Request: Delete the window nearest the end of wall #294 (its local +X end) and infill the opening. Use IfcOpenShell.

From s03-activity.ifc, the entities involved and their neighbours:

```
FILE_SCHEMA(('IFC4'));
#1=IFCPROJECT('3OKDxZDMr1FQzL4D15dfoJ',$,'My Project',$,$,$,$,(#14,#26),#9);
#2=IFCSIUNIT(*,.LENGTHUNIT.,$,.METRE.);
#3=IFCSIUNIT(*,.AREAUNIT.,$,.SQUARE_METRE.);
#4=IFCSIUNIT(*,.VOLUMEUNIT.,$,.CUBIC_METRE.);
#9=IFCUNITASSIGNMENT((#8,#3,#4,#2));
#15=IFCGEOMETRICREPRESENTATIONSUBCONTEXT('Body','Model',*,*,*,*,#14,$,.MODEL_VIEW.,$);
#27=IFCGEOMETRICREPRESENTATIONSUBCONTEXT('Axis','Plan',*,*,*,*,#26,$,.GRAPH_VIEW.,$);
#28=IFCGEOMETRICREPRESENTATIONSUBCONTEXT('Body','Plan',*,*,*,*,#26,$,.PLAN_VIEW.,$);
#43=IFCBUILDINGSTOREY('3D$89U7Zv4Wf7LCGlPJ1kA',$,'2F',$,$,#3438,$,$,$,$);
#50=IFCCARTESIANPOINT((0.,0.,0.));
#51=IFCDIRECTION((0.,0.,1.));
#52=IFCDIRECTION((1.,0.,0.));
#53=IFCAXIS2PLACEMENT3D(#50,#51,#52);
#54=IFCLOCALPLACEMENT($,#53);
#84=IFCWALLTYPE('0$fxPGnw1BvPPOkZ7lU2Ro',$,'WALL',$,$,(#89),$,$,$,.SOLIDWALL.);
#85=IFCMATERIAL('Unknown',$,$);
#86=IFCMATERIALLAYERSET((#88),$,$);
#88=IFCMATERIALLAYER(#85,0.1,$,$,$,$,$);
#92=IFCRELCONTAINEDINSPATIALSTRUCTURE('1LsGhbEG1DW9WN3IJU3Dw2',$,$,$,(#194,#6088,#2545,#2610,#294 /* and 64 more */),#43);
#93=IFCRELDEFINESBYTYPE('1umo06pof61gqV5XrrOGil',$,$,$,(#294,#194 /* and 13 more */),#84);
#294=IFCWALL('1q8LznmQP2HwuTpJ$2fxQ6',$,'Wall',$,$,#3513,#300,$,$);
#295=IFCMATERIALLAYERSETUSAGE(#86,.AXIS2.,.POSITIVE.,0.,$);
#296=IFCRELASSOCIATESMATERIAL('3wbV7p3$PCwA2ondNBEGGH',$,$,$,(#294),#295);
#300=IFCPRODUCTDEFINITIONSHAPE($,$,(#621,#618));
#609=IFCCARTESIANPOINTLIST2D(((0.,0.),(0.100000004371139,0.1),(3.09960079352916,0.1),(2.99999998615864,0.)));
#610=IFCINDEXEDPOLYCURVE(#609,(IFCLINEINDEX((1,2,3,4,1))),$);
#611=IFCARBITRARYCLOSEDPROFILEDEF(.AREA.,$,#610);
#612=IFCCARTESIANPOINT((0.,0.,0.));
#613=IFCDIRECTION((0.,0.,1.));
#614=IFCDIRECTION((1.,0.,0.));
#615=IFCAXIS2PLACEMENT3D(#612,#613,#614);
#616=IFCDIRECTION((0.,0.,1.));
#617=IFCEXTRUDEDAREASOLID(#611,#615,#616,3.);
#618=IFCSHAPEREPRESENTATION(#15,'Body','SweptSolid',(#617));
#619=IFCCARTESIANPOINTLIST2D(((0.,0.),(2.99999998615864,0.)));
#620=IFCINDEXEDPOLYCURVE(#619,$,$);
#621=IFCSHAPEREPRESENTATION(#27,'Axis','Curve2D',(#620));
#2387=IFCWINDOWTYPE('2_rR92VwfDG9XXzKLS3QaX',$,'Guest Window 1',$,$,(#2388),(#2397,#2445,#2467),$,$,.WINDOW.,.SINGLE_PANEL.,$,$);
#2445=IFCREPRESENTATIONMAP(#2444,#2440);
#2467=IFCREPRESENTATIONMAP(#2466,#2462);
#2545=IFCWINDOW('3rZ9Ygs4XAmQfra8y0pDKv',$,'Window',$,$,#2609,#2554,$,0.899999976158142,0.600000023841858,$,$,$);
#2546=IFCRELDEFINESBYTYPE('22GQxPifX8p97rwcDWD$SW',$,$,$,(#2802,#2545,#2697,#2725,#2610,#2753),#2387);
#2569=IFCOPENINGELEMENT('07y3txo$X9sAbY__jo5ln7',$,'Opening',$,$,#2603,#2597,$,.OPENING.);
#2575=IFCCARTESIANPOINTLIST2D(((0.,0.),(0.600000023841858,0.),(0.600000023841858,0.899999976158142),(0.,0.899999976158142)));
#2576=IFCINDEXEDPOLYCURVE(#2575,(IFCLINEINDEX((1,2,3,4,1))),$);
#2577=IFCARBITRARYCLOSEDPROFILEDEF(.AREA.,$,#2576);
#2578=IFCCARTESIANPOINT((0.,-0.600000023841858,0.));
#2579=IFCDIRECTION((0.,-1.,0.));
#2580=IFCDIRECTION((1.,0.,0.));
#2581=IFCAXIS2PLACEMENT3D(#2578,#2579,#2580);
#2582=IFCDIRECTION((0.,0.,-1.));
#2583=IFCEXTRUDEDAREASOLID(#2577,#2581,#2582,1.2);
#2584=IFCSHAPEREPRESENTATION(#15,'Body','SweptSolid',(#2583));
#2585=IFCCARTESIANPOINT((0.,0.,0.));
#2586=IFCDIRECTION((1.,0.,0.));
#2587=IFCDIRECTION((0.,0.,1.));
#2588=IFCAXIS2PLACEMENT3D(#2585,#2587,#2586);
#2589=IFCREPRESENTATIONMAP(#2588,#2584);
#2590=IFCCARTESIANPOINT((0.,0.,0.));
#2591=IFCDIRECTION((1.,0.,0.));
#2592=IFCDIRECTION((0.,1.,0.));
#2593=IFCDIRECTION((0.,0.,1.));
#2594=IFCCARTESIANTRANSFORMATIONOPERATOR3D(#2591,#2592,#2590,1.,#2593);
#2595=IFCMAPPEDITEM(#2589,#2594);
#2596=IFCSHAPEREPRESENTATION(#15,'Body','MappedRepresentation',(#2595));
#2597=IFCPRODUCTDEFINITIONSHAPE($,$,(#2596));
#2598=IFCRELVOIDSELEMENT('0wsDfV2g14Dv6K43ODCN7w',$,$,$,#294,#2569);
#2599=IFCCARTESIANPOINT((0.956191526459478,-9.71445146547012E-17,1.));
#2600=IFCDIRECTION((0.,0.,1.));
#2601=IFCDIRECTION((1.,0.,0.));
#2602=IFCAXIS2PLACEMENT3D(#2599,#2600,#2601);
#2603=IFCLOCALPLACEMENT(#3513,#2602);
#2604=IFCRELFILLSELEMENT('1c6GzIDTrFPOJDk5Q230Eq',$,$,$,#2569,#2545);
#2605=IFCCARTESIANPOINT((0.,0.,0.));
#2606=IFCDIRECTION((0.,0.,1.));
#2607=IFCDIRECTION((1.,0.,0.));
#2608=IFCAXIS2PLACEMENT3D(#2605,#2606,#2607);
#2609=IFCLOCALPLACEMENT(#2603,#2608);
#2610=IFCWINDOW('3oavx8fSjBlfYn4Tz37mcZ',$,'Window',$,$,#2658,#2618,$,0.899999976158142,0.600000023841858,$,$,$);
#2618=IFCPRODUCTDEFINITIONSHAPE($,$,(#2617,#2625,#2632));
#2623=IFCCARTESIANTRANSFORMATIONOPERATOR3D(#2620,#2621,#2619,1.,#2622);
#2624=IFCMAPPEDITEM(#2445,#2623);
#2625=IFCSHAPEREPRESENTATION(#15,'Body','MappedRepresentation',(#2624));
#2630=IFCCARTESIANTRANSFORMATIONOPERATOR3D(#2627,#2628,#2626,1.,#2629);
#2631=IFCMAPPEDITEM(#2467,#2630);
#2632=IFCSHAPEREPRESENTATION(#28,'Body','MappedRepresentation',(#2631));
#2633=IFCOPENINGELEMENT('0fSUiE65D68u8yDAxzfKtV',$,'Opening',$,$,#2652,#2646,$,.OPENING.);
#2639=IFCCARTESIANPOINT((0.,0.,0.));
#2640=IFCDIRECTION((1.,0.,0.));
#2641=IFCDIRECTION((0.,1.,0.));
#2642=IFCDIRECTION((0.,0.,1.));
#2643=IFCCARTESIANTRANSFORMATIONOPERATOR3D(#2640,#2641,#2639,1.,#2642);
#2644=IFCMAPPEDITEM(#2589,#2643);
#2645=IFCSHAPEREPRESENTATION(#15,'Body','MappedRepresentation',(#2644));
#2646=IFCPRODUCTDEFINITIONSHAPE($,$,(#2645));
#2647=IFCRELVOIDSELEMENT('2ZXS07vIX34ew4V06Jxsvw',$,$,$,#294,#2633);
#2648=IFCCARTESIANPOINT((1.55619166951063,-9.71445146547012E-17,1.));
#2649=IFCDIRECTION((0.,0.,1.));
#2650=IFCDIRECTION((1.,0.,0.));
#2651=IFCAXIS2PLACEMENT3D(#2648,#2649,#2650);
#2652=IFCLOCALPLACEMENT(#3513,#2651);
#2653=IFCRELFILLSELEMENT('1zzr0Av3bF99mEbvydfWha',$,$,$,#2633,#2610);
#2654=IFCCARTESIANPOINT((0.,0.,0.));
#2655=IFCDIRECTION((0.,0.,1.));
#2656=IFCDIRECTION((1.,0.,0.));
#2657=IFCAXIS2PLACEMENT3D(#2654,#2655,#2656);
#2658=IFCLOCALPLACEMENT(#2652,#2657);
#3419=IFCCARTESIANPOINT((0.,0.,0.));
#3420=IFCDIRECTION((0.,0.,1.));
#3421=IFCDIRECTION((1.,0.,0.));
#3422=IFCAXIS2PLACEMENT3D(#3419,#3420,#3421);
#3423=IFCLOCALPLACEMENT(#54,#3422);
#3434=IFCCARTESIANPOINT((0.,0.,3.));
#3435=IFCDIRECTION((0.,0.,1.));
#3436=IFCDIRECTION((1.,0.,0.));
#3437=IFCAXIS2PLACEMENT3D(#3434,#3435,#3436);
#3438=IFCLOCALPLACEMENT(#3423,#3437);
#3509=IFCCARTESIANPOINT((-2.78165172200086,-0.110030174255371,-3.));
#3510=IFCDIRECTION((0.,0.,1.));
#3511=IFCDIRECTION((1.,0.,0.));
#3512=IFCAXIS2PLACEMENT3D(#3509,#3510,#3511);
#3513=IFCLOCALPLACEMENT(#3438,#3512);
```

```python
import ifcopenshell
import ifcopenshell.api.feature
import ifcopenshell.api.root
import ifcopenshell.geom
import ifcopenshell.util.shape

model = ifcopenshell.open("s03-activity.ifc")
settings = ifcopenshell.geom.settings()


def volume(element):
    """Net volume in cubic metres, openings subtracted."""
    shape = ifcopenshell.geom.create_shape(settings, element)
    return ifcopenshell.util.shape.get_volume(shape.geometry)


window = model.by_guid("3oavx8fSjBlfYn4Tz37mcZ")
opening = window.FillsVoids[0].RelatingOpeningElement
wall = opening.VoidsElements[0].RelatingBuildingElement
before = volume(wall)

ifcopenshell.api.root.remove_product(model, product=window)
ifcopenshell.api.feature.remove_feature(model, feature=opening)

after = volume(wall)

print(f"wall volume {before:.3f} -> {after:.3f} m3")

model.write("s03-activity_v2.ifc")
```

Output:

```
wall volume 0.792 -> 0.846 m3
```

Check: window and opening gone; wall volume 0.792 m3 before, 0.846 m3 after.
